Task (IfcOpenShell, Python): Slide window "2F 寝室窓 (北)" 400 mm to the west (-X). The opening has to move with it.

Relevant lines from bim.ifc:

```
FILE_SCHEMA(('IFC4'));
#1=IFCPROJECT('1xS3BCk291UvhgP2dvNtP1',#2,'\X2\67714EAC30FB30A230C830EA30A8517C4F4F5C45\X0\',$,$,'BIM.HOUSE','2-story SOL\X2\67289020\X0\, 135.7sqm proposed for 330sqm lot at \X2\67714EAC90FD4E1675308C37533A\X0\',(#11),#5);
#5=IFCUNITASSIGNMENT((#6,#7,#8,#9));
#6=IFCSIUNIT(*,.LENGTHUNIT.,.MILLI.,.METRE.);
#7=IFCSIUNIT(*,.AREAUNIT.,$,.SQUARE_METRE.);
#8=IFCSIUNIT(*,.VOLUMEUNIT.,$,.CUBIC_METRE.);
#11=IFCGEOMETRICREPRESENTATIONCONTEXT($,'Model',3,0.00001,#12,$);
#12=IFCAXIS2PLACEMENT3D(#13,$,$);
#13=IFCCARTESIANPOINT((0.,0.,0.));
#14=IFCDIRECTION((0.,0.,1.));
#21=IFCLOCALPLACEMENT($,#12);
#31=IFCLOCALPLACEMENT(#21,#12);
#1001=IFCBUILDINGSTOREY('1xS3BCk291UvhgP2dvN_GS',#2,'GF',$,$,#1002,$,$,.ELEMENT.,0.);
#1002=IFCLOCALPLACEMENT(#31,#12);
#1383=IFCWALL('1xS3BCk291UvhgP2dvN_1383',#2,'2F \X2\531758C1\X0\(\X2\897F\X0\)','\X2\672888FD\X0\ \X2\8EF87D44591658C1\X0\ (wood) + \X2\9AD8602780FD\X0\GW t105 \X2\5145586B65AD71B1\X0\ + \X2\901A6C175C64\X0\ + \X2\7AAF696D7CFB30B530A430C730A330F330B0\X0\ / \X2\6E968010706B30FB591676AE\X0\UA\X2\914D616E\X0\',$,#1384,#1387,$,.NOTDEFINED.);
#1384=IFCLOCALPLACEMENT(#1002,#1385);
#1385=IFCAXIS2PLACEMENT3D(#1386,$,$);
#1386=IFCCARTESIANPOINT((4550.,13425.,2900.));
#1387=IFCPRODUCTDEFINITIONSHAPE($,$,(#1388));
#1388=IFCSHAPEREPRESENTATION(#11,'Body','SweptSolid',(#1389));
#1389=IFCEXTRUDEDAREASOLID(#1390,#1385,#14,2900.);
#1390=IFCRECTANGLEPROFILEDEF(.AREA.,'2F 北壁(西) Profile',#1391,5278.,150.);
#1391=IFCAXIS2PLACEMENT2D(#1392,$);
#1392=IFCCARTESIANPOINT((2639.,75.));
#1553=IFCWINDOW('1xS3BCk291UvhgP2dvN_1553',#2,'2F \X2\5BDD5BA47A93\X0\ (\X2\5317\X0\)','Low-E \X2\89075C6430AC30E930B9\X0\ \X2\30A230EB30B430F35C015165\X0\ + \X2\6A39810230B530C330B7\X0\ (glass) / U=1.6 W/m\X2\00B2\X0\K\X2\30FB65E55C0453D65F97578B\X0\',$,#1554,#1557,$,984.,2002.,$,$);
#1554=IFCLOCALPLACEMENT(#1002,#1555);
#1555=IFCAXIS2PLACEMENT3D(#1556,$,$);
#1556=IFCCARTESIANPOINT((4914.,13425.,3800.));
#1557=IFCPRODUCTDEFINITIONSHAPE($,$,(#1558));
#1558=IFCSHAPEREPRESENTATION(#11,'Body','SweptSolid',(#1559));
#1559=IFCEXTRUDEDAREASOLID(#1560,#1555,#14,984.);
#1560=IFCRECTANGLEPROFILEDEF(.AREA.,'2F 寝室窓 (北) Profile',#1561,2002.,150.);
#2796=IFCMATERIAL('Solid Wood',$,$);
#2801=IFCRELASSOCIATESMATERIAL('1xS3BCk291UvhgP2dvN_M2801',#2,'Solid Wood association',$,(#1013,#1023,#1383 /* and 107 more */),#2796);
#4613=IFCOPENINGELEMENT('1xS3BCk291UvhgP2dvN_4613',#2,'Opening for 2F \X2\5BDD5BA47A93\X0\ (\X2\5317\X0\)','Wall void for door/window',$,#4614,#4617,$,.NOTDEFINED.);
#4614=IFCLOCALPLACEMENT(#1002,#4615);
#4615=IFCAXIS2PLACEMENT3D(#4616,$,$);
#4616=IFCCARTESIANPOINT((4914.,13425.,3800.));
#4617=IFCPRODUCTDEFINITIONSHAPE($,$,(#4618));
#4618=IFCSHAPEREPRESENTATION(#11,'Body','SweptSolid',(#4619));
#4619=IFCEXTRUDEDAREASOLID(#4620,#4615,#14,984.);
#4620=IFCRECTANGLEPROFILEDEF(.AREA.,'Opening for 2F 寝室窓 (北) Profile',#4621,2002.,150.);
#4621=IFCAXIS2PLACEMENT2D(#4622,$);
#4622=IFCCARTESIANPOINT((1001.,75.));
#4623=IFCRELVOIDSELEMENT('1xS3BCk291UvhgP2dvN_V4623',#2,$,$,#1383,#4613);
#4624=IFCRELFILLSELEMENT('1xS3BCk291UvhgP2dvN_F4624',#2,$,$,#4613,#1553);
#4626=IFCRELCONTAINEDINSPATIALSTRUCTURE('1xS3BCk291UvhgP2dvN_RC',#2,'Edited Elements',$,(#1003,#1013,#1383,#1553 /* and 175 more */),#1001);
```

```python
import ifcopenshell
import ifcopenshell.api.geometry
import ifcopenshell.util.placement
import ifcopenshell.util.unit

model = ifcopenshell.open("bim.ifc")
unit_scale = ifcopenshell.util.unit.calculate_unit_scale(model)

window = model.by_guid("1xS3BCk291UvhgP2dvN_1553")
opening = window.FillsVoids[0].RelatingOpeningElement
wall = opening.VoidsElements[0].RelatingBuildingElement

wall_matrix = ifcopenshell.util.placement.get_local_placement(wall.ObjectPlacement)
shift = wall_matrix[:3, 0] * -0.4 / unit_scale
before = ifcopenshell.util.placement.get_local_placement(window.ObjectPlacement)[:3, 3].copy()

# The window is not placed relative to its opening, so move both.
for product in (opening, window):
    matrix = ifcopenshell.util.placement.get_local_placement(product.ObjectPlacement)
    matrix[:3, 3] += shift
    ifcopenshell.api.geometry.edit_object_placement(model, product=product, matrix=matrix, is_si=False)

after = ifcopenshell.util.placement.get_local_placement(window.ObjectPlacement)[:3, 3]
print("window moved by", (after - before).round(3) + 0.0)

model.write("bim-out.ifc")
```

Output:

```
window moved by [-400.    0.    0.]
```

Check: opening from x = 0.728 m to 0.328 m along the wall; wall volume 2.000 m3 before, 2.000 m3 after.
